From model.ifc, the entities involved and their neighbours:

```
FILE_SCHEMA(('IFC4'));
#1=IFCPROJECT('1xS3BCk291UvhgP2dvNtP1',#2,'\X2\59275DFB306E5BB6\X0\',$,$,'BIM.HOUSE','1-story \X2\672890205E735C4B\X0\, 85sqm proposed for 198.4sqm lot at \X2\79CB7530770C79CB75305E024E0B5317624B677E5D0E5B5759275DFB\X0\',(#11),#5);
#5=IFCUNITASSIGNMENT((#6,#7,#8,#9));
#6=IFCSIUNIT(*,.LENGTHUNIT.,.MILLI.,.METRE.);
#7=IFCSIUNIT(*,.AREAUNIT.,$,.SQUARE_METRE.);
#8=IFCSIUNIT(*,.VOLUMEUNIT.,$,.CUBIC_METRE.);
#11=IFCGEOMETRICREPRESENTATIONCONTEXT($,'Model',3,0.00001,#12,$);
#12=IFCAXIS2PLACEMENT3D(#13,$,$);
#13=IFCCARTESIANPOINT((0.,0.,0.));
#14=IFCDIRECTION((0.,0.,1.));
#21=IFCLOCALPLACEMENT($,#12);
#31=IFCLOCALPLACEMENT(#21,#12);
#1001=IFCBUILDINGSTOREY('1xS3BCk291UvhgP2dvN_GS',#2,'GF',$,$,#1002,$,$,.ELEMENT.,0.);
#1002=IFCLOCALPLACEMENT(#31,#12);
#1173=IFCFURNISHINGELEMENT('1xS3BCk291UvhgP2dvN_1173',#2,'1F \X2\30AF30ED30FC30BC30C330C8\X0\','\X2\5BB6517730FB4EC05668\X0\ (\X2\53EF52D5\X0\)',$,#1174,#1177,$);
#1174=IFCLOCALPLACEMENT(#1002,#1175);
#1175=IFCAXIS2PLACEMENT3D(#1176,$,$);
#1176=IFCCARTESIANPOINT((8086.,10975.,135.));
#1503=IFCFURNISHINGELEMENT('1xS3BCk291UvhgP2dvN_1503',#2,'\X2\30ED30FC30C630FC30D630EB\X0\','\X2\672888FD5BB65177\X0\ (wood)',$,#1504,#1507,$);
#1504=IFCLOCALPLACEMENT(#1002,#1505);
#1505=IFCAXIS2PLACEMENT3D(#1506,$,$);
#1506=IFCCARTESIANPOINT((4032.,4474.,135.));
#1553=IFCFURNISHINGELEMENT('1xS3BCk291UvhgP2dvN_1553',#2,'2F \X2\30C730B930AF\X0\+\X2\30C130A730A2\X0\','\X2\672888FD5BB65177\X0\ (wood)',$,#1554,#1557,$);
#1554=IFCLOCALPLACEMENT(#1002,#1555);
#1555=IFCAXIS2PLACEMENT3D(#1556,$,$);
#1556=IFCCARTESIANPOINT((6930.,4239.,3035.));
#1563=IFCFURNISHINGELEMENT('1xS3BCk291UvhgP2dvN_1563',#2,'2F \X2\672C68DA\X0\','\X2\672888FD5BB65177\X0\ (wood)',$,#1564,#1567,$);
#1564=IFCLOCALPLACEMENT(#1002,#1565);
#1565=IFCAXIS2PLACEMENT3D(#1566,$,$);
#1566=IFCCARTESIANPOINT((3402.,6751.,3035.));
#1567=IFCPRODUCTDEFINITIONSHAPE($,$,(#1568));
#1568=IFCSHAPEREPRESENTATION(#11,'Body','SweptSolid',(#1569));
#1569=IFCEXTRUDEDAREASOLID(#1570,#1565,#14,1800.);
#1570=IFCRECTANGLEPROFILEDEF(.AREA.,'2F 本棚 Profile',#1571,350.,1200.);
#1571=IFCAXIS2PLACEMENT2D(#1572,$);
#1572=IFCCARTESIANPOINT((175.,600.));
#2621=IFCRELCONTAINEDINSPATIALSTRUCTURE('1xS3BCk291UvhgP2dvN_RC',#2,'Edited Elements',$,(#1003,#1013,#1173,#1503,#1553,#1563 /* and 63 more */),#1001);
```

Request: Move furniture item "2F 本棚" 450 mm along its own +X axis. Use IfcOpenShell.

```python
import ifcopenshell
import ifcopenshell.api.geometry
import ifcopenshell.util.placement
import ifcopenshell.util.unit

model = ifcopenshell.open("model.ifc")
unit_scale = ifcopenshell.util.unit.calculate_unit_scale(model)

item = model.by_guid("1xS3BCk291UvhgP2dvN_1563")
matrix = ifcopenshell.util.placement.get_local_placement(item.ObjectPlacement)
matrix[:3, 3] += matrix[:3, 0] * 0.45 / unit_scale
ifcopenshell.api.geometry.edit_object_placement(model, product=item, matrix=matrix, is_si=False)

print(ifcopenshell.util.placement.get_local_placement(item.ObjectPlacement).round(3) + 0.0)

model.write("model_rev.ifc")
```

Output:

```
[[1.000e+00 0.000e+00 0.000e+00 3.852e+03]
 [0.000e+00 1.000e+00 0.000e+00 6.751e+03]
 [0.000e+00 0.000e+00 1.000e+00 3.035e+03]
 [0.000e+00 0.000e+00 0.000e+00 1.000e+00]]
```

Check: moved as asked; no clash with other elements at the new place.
